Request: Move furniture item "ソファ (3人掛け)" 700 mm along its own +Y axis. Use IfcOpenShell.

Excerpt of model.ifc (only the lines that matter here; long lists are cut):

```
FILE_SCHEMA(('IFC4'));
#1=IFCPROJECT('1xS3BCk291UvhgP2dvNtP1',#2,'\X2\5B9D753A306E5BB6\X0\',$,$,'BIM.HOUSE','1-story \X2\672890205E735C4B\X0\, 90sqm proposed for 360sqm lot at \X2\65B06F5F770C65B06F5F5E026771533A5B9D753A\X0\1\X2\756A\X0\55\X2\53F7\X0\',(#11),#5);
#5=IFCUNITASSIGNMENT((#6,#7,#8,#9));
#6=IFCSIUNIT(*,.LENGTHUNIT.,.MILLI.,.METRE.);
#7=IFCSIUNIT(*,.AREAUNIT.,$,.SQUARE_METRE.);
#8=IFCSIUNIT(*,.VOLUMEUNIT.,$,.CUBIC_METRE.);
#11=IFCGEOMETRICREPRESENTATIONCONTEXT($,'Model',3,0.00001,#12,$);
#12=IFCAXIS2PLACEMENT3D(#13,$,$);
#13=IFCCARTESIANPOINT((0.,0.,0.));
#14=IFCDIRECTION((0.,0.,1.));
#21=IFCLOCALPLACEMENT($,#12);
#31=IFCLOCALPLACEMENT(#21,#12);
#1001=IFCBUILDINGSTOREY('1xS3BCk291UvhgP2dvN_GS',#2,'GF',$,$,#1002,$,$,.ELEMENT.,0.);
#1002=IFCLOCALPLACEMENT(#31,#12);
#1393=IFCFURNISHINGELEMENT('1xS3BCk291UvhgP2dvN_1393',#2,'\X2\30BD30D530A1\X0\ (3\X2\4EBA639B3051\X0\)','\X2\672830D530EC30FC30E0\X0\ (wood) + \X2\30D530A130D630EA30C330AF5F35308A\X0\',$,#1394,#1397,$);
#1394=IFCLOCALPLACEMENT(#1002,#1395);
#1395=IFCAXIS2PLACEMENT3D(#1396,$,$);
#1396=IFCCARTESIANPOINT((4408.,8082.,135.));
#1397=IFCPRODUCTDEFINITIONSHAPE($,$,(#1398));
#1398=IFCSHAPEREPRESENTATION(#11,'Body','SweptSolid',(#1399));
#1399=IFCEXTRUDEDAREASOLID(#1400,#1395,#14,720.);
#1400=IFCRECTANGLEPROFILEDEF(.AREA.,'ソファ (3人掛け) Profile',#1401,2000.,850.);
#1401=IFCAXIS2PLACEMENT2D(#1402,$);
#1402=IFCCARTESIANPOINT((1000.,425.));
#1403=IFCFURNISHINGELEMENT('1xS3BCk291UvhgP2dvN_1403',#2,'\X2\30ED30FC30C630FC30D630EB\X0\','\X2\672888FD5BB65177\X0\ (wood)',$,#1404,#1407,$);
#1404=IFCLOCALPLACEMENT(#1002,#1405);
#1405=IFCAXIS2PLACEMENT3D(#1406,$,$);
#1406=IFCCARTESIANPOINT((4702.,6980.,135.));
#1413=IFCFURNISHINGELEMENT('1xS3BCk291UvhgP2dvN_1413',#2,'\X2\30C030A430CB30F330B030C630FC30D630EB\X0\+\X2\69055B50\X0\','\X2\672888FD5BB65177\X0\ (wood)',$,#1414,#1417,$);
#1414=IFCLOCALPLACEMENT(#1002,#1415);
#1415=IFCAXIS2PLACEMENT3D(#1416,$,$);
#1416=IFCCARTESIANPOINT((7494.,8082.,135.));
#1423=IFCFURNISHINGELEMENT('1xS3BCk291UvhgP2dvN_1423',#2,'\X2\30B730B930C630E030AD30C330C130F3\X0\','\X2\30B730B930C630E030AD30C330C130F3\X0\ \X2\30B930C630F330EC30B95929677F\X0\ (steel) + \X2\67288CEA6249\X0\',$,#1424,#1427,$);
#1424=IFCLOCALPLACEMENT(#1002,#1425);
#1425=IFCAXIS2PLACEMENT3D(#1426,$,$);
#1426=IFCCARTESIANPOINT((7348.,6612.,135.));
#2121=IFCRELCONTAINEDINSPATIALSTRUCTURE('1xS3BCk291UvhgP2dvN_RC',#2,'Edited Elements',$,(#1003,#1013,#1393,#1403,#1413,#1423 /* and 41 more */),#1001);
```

```python
import ifcopenshell
import ifcopenshell.api.geometry
import ifcopenshell.util.placement

model = ifcopenshell.open("model.ifc")

item = model.by_guid("1xS3BCk291UvhgP2dvN_1393")
matrix = ifcopenshell.util.placement.get_local_placement(item.ObjectPlacement)
matrix[:3, 3] += matrix[:3, 1] * 700.0
ifcopenshell.api.geometry.edit_object_placement(model, product=item, matrix=matrix, is_si=False)

print(ifcopenshell.util.placement.get_local_placement(item.ObjectPlacement).round(3) + 0.0)

model.write("model_v2.ifc")
```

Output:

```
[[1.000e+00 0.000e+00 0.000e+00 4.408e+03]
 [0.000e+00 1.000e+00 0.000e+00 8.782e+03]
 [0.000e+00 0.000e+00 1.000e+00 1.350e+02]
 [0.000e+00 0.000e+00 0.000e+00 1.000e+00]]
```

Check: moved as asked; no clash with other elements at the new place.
